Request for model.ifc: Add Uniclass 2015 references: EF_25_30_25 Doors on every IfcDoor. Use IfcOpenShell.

First a look at what the model holds.

```python
import ifcopenshell

model = ifcopenshell.open("model.ifc")
print(model.schema)
print("classifications:", [c.Name for c in model.by_type("IfcClassification")])
for ifc_class in ("IfcDoor", "IfcRoof", "IfcStair", "IfcWall", "IfcWindow"):
    print(ifc_class, len(model.by_type(ifc_class)))
```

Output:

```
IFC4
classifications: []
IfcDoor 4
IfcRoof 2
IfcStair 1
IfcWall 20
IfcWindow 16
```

```python
import ifcopenshell
import ifcopenshell.api.classification

model = ifcopenshell.open("model.ifc")

system = ifcopenshell.api.classification.add_classification(model, classification="Uniclass 2015")

codes = {
    "IfcDoor": ("EF_25_30_25", "Doors"),
}
for ifc_class, (code, name) in codes.items():
    products = model.by_type(ifc_class)
    ifcopenshell.api.classification.add_reference(
        model, products=products, classification=system, identification=code, name=name
    )
    print(code, len(products))

model.write("model_edited.ifc")
```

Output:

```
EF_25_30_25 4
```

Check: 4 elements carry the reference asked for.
